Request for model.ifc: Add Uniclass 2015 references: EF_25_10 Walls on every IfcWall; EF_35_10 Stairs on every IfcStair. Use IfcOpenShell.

First a look at what the model holds.

```python
import ifcopenshell

model = ifcopenshell.open("model.ifc")
print(model.schema)
print("classifications:", [c.Name for c in model.by_type("IfcClassification")])
for ifc_class in ("IfcDoor", "IfcRoof", "IfcStair", "IfcWall", "IfcWindow"):
    print(ifc_class, len(model.by_type(ifc_class)))
```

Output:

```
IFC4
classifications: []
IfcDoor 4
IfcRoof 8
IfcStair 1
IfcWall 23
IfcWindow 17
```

```python
import ifcopenshell
import ifcopenshell.api.classification

model = ifcopenshell.open("model.ifc")

system = ifcopenshell.api.classification.add_classification(model, classification="Uniclass 2015")

codes = {
    "IfcWall": ("EF_25_10", "Walls"),
    "IfcStair": ("EF_35_10", "Stairs"),
}
for ifc_class, (code, name) in codes.items():
    products = model.by_type(ifc_class)
    ifcopenshell.api.classification.add_reference(
        model, products=products, classification=system, identification=code, name=name
    )
    print(code, len(products))

model.write("model-out.ifc")
```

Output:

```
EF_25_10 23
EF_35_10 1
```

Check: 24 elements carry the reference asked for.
